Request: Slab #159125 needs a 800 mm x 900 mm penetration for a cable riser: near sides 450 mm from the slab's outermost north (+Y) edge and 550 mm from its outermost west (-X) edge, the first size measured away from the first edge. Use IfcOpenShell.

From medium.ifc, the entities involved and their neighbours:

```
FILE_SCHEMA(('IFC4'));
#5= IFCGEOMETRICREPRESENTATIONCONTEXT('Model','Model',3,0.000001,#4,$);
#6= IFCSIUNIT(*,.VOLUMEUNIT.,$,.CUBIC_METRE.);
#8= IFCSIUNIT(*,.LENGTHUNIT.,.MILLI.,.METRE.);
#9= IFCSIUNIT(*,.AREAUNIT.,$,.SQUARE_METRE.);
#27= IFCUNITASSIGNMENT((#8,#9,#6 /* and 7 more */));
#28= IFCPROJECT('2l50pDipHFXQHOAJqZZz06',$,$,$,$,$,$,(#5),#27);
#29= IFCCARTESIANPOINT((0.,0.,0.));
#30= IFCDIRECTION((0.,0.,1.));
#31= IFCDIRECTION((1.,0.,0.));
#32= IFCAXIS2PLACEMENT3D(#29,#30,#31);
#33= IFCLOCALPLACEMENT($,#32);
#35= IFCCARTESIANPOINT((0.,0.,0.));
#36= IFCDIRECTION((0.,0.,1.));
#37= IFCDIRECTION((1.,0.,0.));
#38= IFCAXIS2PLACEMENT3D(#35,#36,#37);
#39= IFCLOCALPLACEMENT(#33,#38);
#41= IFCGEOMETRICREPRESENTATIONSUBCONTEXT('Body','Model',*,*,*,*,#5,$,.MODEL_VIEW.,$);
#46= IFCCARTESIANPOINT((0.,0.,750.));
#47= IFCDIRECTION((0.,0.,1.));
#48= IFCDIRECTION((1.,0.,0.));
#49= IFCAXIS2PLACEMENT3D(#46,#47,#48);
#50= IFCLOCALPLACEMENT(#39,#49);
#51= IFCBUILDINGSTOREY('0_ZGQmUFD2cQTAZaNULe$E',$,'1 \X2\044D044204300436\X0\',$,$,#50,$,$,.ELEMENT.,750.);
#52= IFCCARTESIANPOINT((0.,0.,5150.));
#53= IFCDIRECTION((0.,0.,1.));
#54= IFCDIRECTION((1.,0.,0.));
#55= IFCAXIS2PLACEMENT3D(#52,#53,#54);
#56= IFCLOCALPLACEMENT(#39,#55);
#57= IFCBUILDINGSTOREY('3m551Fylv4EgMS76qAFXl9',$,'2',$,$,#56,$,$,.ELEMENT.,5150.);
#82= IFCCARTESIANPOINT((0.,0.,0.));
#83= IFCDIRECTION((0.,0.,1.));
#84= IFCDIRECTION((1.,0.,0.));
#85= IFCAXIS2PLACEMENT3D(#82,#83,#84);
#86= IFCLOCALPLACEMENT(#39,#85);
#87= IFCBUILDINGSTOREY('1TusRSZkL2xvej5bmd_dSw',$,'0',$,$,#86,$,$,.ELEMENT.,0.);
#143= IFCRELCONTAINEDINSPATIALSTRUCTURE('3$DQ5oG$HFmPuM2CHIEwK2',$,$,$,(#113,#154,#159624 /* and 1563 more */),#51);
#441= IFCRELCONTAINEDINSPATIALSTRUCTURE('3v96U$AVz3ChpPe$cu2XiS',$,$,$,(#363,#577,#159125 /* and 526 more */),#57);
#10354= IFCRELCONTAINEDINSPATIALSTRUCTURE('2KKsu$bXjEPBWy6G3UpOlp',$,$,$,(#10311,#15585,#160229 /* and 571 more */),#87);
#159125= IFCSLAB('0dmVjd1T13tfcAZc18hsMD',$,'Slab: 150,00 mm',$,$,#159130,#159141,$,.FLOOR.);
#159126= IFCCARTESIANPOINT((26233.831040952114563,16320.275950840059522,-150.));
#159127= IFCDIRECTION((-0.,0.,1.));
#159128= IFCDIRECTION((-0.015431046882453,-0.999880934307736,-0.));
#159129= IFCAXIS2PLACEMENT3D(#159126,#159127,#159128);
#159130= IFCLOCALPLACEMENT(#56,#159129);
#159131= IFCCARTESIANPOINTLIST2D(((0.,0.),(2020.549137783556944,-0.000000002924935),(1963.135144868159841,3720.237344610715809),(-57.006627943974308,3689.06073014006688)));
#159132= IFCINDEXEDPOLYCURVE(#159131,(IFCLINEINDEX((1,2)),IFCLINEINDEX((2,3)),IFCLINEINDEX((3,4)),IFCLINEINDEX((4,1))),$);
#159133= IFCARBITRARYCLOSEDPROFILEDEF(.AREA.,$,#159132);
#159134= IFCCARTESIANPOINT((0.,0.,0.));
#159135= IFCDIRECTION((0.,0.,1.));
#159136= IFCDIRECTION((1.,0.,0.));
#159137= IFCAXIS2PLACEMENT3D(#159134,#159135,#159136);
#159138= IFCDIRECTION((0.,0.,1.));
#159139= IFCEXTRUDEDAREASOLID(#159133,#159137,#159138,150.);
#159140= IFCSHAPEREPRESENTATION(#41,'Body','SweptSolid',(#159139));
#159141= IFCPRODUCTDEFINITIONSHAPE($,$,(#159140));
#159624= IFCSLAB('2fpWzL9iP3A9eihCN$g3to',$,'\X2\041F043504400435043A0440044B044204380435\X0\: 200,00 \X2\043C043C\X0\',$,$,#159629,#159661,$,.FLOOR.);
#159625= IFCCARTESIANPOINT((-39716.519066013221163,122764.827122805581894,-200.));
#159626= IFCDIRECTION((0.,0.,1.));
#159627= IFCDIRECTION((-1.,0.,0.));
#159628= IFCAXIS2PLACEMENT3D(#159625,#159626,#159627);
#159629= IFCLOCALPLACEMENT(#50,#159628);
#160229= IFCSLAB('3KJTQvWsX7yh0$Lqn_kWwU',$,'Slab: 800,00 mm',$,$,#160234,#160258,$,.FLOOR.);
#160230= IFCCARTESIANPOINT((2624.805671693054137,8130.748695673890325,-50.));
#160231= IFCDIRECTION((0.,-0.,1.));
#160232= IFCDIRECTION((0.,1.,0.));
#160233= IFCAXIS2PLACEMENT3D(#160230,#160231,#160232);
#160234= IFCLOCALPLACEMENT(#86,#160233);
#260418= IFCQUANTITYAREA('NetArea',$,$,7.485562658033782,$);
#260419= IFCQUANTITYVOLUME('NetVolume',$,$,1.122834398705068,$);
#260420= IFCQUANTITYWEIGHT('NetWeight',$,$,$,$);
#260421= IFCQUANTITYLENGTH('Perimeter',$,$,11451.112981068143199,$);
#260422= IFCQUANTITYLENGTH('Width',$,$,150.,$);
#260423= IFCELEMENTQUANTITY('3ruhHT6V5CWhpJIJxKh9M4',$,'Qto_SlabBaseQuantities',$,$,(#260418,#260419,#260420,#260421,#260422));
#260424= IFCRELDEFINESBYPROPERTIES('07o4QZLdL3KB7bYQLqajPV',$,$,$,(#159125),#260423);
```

```python
import numpy as np
import ifcopenshell
import ifcopenshell.api.feature
import ifcopenshell.api.geometry
import ifcopenshell.api.pset
import ifcopenshell.api.root
import ifcopenshell.geom
import ifcopenshell.util.element
import ifcopenshell.util.placement
import ifcopenshell.util.representation
import ifcopenshell.util.shape
import ifcopenshell.util.unit

model = ifcopenshell.open("medium.ifc")
unit_scale = ifcopenshell.util.unit.calculate_unit_scale(model)
area_scale = ifcopenshell.util.unit.calculate_unit_scale(model, "AREAUNIT")
volume_scale = ifcopenshell.util.unit.calculate_unit_scale(model, "VOLUMEUNIT")
settings = ifcopenshell.geom.settings()


def volume(element):
    """Net volume in cubic metres, openings subtracted."""
    shape = ifcopenshell.geom.create_shape(settings, element)
    return ifcopenshell.util.shape.get_volume(shape.geometry)


slab = model.by_id(159125)
before = volume(slab)

# Extent in the slab's own axes, in metres. The edges named are its -X and -Y sides.
slab_shape = ifcopenshell.geom.create_shape(settings, slab)
vertices = ifcopenshell.util.shape.get_vertices(slab_shape.geometry)
x_min, y_min, bottom = vertices.min(axis=0)
top = vertices[:, 2].max()

opening = ifcopenshell.api.root.create_entity(model, ifc_class="IfcOpeningElement", name="Cable riser opening", predefined_type="OPENING")
context = ifcopenshell.util.representation.get_context(model, "Model", "Body", "MODEL_VIEW")
width, depth = 0.8, 0.9
outline = [(0.0, 0.0), (width, 0.0), (width, depth), (0.0, depth), (0.0, 0.0)]
# Overshoot both faces by 50 mm so the cut is clean.
shape = ifcopenshell.api.geometry.add_slab_representation(
    model, context=context, depth=top - bottom + 0.1, polyline=outline
)
ifcopenshell.api.geometry.assign_representation(model, product=opening, representation=shape)

matrix = ifcopenshell.util.placement.get_local_placement(slab.ObjectPlacement)
matrix[:, 3] = matrix @ np.append(np.array([x_min + 0.45, y_min + 0.55, bottom - 0.05]) / unit_scale, 1.0)
ifcopenshell.api.geometry.edit_object_placement(model, product=opening, matrix=matrix, is_si=False)
ifcopenshell.api.feature.add_feature(model, feature=opening, element=slab)

after = volume(slab)

# Update the slab's stored quantities.
qto = model.by_id(ifcopenshell.util.element.get_pset(slab, "Qto_SlabBaseQuantities", should_inherit=False)["id"])
ifcopenshell.api.pset.edit_qto(model, qto=qto, properties={
    "NetArea": after / (top - bottom) / area_scale,
    "NetVolume": after / volume_scale,
})

print(f"slab volume {before:.3f} -> {after:.3f} m3")

model.write("medium_edited.ifc")
```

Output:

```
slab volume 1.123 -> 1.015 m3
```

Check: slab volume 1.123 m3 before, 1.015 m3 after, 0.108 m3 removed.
